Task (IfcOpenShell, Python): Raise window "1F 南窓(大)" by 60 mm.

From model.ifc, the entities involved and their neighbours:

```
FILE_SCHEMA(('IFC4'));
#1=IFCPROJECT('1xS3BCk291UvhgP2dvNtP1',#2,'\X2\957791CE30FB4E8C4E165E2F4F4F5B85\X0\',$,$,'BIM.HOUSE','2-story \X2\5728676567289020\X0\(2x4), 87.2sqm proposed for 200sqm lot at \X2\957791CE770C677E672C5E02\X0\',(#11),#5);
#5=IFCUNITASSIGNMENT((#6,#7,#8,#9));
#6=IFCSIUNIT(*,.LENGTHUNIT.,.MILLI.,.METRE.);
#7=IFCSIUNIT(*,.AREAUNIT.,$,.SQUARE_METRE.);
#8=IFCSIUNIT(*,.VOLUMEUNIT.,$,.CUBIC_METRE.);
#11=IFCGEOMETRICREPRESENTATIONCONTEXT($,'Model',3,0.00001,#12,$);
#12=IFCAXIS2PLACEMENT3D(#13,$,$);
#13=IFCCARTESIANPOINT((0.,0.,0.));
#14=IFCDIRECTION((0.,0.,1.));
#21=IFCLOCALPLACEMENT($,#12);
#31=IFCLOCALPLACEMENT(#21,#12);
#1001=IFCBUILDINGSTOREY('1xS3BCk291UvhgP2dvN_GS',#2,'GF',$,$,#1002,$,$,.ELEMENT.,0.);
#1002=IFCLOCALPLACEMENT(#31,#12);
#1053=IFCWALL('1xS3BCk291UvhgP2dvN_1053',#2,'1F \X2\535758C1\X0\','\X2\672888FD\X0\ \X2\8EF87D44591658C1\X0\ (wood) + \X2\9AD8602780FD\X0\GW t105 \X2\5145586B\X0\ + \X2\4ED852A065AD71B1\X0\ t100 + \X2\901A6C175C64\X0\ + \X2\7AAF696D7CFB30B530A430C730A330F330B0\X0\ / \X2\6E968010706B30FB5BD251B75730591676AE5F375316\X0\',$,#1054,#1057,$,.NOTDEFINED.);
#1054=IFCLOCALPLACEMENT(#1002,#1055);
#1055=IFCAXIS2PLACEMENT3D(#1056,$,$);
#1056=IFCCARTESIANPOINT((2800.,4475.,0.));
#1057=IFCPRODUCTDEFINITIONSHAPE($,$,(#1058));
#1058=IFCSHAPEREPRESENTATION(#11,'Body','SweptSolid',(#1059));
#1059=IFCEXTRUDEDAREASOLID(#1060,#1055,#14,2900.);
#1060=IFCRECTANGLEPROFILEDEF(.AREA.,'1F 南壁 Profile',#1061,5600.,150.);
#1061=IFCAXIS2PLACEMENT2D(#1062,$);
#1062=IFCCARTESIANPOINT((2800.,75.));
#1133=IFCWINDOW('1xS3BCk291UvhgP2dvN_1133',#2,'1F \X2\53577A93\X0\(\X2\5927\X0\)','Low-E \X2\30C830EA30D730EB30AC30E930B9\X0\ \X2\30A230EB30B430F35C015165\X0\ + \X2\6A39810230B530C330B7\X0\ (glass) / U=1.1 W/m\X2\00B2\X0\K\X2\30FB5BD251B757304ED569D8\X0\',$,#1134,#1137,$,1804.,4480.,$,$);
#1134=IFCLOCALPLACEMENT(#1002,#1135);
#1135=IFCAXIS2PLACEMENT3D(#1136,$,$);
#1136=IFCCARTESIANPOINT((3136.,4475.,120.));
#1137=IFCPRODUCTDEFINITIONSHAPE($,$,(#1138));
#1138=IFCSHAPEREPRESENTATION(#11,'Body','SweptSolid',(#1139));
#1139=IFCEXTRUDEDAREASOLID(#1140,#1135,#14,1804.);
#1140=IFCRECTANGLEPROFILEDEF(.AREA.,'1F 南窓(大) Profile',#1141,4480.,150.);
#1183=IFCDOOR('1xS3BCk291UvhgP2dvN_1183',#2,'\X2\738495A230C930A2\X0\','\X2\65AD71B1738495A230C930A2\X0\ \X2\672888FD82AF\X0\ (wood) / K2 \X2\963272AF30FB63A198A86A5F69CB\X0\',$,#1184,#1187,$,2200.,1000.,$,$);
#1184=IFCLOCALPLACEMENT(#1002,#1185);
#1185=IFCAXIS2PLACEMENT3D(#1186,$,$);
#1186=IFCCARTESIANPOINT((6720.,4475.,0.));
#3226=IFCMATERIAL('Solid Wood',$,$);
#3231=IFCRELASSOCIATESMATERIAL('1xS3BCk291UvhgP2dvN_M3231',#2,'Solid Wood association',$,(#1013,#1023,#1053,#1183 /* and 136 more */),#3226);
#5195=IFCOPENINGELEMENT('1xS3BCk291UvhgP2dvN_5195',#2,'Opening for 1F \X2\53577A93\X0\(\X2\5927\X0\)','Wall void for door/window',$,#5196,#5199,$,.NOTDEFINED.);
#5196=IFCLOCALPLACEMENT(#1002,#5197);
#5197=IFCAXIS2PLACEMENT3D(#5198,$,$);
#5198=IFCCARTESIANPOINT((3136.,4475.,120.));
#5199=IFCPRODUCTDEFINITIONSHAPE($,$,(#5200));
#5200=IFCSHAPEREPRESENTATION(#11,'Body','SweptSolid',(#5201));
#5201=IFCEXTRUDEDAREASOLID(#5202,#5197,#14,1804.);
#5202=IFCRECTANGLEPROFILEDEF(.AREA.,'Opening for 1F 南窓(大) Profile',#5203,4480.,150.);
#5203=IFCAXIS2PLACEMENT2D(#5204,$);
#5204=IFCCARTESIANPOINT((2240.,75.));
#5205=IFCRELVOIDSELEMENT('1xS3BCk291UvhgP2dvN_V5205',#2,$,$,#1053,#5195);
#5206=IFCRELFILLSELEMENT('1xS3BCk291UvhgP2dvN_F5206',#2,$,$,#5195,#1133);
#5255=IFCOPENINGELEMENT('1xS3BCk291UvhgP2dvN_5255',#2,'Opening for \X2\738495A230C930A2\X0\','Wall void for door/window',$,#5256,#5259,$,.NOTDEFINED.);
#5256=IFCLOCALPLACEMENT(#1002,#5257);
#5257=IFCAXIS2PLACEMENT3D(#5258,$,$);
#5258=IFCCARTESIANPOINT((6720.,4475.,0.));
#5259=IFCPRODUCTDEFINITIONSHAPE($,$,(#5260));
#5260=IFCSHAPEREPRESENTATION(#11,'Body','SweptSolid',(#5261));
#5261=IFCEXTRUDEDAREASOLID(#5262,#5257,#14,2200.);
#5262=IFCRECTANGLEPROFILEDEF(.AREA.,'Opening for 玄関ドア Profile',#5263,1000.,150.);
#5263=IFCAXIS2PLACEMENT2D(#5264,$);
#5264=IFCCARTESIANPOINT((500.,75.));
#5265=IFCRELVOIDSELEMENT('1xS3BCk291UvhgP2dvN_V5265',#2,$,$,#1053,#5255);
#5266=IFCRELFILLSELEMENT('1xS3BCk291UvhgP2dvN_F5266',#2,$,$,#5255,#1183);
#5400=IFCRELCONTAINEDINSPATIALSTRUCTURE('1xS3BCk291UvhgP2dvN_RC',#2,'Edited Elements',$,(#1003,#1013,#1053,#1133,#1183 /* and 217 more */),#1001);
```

```python
import numpy as np
import ifcopenshell
import ifcopenshell.api.geometry
import ifcopenshell.util.placement
import ifcopenshell.util.unit

model = ifcopenshell.open("model.ifc")
unit_scale = ifcopenshell.util.unit.calculate_unit_scale(model)

window = model.by_guid("1xS3BCk291UvhgP2dvN_1133")
opening = window.FillsVoids[0].RelatingOpeningElement
dz = 0.06 / unit_scale

shift = np.array([0.0, 0.0, dz])
# The window is not placed relative to its opening, so move both.
for product in (opening, window):
    matrix = ifcopenshell.util.placement.get_local_placement(product.ObjectPlacement)
    matrix[:3, 3] += shift
    ifcopenshell.api.geometry.edit_object_placement(model, product=product, matrix=matrix, is_si=False)

print(f"moved by {dz * unit_scale:+.3f} m")

model.write("model_rev.ifc")
```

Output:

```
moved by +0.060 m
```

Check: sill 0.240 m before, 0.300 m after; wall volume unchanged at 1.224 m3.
